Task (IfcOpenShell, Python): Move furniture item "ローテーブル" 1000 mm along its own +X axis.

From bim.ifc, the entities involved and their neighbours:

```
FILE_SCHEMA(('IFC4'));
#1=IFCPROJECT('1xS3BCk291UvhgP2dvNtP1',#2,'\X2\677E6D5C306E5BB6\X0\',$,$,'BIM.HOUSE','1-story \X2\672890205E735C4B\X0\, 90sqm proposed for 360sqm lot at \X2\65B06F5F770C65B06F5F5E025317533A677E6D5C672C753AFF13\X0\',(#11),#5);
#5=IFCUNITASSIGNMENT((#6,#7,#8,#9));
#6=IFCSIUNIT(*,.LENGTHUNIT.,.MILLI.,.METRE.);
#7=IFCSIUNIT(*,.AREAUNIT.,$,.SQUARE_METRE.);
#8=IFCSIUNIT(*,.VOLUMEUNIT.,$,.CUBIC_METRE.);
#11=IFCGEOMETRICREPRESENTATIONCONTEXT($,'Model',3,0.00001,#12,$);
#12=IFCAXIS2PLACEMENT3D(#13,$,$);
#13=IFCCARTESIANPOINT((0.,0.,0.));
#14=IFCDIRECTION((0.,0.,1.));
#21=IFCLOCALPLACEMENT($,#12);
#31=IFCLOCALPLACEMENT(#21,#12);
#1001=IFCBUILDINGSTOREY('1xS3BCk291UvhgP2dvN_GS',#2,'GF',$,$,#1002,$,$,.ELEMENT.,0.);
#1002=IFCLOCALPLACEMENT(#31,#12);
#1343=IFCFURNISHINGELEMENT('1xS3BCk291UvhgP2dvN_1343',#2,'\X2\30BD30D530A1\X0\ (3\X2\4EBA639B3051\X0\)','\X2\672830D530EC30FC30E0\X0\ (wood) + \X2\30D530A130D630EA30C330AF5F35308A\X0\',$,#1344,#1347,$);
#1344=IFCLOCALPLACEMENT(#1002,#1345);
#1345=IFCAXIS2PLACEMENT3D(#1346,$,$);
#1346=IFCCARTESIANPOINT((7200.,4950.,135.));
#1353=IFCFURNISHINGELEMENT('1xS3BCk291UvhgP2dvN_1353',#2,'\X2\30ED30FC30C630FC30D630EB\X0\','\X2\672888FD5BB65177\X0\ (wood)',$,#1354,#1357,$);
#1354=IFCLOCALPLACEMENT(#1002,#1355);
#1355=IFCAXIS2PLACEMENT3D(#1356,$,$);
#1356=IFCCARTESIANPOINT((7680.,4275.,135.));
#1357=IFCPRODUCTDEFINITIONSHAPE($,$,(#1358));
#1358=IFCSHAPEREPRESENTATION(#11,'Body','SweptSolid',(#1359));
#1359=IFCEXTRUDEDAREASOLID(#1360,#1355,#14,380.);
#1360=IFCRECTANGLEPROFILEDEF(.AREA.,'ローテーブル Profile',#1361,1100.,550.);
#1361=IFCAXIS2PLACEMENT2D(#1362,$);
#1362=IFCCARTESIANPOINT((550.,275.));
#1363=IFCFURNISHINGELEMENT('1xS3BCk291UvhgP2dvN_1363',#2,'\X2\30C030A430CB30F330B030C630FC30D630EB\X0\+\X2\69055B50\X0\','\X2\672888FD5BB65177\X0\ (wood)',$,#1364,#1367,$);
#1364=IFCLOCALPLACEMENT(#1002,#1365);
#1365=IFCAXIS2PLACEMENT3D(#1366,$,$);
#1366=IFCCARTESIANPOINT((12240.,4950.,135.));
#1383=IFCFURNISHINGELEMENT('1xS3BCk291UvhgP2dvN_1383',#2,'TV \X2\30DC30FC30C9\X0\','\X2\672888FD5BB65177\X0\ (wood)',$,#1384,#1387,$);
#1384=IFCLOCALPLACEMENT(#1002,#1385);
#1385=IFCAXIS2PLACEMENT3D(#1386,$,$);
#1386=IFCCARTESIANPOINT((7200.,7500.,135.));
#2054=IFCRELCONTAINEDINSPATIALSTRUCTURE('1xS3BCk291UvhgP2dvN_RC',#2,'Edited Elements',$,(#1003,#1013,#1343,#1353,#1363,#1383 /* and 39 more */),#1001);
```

```python
import ifcopenshell
import ifcopenshell.api.geometry
import ifcopenshell.util.placement

model = ifcopenshell.open("bim.ifc")

item = model.by_guid("1xS3BCk291UvhgP2dvN_1353")
matrix = ifcopenshell.util.placement.get_local_placement(item.ObjectPlacement)
matrix[:3, 3] += matrix[:3, 0] * 1000.0
ifcopenshell.api.geometry.edit_object_placement(model, product=item, matrix=matrix, is_si=False)

print(ifcopenshell.util.placement.get_local_placement(item.ObjectPlacement).round(3) + 0.0)

model.write("bim_rev.ifc")
```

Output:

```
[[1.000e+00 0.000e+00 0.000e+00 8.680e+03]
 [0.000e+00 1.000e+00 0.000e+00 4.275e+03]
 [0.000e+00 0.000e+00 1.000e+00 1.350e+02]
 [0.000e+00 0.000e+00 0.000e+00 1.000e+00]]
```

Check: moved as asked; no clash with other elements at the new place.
